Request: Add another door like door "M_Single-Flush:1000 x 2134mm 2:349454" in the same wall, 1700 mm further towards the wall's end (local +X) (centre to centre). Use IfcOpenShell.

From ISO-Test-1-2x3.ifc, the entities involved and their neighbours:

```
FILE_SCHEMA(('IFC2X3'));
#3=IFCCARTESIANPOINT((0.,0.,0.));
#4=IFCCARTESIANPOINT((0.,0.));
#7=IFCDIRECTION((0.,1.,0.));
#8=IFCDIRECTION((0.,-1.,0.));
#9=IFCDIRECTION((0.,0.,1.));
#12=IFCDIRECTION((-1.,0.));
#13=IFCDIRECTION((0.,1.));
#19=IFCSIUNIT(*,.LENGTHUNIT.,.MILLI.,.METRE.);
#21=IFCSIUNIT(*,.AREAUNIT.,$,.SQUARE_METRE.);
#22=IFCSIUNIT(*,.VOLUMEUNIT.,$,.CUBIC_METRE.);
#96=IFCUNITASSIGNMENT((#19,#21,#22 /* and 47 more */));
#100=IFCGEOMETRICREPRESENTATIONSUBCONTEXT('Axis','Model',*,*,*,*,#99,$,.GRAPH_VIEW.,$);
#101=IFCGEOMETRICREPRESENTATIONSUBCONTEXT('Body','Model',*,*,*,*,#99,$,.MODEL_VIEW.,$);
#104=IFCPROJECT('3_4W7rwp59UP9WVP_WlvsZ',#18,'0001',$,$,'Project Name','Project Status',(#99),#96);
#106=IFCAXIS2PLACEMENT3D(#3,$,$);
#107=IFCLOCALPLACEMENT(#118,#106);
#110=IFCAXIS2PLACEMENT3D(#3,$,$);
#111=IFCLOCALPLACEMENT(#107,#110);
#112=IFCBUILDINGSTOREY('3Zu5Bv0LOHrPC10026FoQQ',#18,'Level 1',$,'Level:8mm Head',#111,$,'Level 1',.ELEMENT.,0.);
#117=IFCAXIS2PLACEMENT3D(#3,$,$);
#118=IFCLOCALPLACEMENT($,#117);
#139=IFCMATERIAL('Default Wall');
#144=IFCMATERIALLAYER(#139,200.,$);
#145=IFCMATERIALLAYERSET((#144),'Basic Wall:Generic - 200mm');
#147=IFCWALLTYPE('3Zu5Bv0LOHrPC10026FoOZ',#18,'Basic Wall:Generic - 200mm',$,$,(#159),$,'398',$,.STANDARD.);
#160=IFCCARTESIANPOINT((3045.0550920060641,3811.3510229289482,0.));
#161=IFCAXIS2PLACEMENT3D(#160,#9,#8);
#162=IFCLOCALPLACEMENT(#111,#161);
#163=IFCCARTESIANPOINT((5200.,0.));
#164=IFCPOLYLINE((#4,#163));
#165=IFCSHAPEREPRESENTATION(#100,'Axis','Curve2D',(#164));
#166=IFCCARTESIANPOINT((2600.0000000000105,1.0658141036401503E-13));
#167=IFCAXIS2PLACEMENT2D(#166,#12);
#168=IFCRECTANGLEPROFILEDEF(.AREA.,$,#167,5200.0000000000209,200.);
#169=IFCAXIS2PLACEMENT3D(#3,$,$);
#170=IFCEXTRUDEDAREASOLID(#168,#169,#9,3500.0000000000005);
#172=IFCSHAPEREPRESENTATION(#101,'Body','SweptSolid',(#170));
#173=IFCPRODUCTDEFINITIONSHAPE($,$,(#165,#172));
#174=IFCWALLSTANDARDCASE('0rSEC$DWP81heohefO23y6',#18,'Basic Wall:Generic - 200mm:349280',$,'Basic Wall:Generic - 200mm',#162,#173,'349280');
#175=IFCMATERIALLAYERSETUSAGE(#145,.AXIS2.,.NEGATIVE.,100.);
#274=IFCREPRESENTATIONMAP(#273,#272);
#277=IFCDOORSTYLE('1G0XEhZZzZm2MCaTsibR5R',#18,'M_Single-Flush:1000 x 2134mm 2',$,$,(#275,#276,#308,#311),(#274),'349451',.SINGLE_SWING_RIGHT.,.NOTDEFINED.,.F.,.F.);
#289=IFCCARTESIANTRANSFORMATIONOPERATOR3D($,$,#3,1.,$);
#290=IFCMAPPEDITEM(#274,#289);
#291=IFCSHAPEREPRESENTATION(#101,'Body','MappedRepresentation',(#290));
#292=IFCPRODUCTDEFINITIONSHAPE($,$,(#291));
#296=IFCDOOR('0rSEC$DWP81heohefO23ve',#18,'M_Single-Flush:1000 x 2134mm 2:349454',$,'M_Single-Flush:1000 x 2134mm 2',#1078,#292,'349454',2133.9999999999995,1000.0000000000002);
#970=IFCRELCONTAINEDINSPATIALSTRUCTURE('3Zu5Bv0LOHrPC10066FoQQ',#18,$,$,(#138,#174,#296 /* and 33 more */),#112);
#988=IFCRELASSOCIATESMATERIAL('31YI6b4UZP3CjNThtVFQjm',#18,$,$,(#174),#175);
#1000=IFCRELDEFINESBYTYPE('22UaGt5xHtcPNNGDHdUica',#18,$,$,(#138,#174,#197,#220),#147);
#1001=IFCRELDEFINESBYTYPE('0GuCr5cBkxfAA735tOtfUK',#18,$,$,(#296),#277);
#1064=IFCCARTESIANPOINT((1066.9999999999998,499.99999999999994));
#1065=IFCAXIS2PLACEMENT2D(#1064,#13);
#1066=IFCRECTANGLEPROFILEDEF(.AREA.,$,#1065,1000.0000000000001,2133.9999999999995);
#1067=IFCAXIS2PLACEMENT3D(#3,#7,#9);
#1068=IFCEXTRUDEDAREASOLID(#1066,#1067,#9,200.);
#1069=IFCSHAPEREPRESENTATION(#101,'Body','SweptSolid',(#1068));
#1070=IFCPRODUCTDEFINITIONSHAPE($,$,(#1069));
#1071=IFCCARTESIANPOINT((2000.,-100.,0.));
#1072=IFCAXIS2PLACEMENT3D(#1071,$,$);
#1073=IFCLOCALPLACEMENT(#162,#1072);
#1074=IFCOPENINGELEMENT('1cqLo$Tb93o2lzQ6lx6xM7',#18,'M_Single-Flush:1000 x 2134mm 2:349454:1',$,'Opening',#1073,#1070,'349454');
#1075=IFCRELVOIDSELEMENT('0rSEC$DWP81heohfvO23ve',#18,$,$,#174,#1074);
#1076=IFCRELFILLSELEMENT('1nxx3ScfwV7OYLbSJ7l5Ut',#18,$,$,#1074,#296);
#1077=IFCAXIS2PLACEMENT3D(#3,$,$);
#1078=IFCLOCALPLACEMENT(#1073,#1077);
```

```python
import ifcopenshell
import ifcopenshell.api.feature
import ifcopenshell.api.geometry
import ifcopenshell.api.root
import ifcopenshell.geom
import ifcopenshell.util.element
import ifcopenshell.util.placement
import ifcopenshell.util.shape

model = ifcopenshell.open("ISO-Test-1-2x3.ifc")
settings = ifcopenshell.geom.settings()


def volume(element):
    """Net volume in cubic metres, openings subtracted."""
    shape = ifcopenshell.geom.create_shape(settings, element)
    return ifcopenshell.util.shape.get_volume(shape.geometry)


def reuse_history(source, copy):
    """copy_class also copies each property set's owner history, people and application; keep the originals."""
    for rel in copy.IsDefinedBy:
        if rel.is_a("IfcRelDefinesByProperties") and (history := rel.RelatingPropertyDefinition.OwnerHistory):
            rel.RelatingPropertyDefinition.OwnerHistory = source.OwnerHistory
            ifcopenshell.util.element.remove_deep2(model, history)


door = model.by_id(296)
opening = door.FillsVoids[0].RelatingOpeningElement
wall = opening.VoidsElements[0].RelatingBuildingElement
before = volume(wall)
shift = ifcopenshell.util.placement.get_local_placement(wall.ObjectPlacement)[:3, 0] * 1700.0

# copy_class copies the void relationship, type, container and properties, but no geometry.
new_opening = ifcopenshell.api.root.copy_class(model, product=opening)
new_opening.Representation = ifcopenshell.util.element.copy_deep(
    model, opening.Representation, exclude=["IfcGeometricRepresentationContext", "IfcRepresentationMap"]
)
new_opening.Name = "M_Single-Flush:1000 x 2134mm 2"
new_opening.Tag = None
new_door = ifcopenshell.api.root.copy_class(model, product=door)
new_door.Representation = ifcopenshell.util.element.copy_deep(
    model, door.Representation, exclude=["IfcGeometricRepresentationContext", "IfcRepresentationMap"]
)
new_door.Name = "M_Single-Flush:1000 x 2134mm 2"
new_door.Tag = None
reuse_history(door, new_door)
fills = ifcopenshell.api.feature.add_filling(model, opening=new_opening, element=new_door)
fills.OwnerHistory = new_door.OwnerHistory  # required in IFC2X3

for old, new in ((opening, new_opening), (door, new_door)):
    matrix = ifcopenshell.util.placement.get_local_placement(old.ObjectPlacement)
    matrix[:3, 3] += shift
    ifcopenshell.api.geometry.edit_object_placement(model, product=new, matrix=matrix, is_si=False)

after = volume(wall)

print(f"wall volume {before:.3f} -> {after:.3f} m3")

model.write("ISO-Test-1-2x3_rev.ifc")
```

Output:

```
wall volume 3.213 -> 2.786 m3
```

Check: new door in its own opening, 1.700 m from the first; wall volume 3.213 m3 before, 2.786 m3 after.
